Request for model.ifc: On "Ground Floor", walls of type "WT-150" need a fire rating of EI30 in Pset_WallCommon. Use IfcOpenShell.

First a look at what the model holds.

```python
import ifcopenshell
import ifcopenshell.util.element

model = ifcopenshell.open("model.ifc")
print(model.schema)
storey = next(s for s in model.by_type("IfcBuildingStorey") if s.Name == "Ground Floor")
walls = [e for e in ifcopenshell.util.element.get_decomposition(storey) if e.is_a("IfcWall")]
seen = {}
for e in walls:
    element_type = ifcopenshell.util.element.get_type(e)
    key = (element_type.Name if element_type != e and element_type else None, ifcopenshell.util.element.get_pset(e, "Pset_WallCommon", "FireRating"))
    seen[key] = seen.get(key, 0) + 1
for (name, value), count in sorted(seen.items(), key=str):
    print(count, "x", name, "|", value)
```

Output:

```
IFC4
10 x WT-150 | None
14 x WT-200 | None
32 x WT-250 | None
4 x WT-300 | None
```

```python
import ifcopenshell
import ifcopenshell.api.pset
import ifcopenshell.util.element

model = ifcopenshell.open("model.ifc")

storey = next(s for s in model.by_type("IfcBuildingStorey") if s.Name == "Ground Floor")
walls = [e for e in ifcopenshell.util.element.get_decomposition(storey) if e.is_a("IfcWall")]

count = 0
for e in walls:
    element_type = ifcopenshell.util.element.get_type(e)
    if element_type in (None, e) or element_type.Name != "WT-150":
        continue
    # add_pset returns the element's existing set when there is one.
    pset = ifcopenshell.api.pset.add_pset(model, product=e, name="Pset_WallCommon")
    ifcopenshell.api.pset.edit_pset(model, pset=pset, properties={"FireRating": "EI30"})
    count += 1

print(count, "walls updated")

model.write("model_v2.ifc")
```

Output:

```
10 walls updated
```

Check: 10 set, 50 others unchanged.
